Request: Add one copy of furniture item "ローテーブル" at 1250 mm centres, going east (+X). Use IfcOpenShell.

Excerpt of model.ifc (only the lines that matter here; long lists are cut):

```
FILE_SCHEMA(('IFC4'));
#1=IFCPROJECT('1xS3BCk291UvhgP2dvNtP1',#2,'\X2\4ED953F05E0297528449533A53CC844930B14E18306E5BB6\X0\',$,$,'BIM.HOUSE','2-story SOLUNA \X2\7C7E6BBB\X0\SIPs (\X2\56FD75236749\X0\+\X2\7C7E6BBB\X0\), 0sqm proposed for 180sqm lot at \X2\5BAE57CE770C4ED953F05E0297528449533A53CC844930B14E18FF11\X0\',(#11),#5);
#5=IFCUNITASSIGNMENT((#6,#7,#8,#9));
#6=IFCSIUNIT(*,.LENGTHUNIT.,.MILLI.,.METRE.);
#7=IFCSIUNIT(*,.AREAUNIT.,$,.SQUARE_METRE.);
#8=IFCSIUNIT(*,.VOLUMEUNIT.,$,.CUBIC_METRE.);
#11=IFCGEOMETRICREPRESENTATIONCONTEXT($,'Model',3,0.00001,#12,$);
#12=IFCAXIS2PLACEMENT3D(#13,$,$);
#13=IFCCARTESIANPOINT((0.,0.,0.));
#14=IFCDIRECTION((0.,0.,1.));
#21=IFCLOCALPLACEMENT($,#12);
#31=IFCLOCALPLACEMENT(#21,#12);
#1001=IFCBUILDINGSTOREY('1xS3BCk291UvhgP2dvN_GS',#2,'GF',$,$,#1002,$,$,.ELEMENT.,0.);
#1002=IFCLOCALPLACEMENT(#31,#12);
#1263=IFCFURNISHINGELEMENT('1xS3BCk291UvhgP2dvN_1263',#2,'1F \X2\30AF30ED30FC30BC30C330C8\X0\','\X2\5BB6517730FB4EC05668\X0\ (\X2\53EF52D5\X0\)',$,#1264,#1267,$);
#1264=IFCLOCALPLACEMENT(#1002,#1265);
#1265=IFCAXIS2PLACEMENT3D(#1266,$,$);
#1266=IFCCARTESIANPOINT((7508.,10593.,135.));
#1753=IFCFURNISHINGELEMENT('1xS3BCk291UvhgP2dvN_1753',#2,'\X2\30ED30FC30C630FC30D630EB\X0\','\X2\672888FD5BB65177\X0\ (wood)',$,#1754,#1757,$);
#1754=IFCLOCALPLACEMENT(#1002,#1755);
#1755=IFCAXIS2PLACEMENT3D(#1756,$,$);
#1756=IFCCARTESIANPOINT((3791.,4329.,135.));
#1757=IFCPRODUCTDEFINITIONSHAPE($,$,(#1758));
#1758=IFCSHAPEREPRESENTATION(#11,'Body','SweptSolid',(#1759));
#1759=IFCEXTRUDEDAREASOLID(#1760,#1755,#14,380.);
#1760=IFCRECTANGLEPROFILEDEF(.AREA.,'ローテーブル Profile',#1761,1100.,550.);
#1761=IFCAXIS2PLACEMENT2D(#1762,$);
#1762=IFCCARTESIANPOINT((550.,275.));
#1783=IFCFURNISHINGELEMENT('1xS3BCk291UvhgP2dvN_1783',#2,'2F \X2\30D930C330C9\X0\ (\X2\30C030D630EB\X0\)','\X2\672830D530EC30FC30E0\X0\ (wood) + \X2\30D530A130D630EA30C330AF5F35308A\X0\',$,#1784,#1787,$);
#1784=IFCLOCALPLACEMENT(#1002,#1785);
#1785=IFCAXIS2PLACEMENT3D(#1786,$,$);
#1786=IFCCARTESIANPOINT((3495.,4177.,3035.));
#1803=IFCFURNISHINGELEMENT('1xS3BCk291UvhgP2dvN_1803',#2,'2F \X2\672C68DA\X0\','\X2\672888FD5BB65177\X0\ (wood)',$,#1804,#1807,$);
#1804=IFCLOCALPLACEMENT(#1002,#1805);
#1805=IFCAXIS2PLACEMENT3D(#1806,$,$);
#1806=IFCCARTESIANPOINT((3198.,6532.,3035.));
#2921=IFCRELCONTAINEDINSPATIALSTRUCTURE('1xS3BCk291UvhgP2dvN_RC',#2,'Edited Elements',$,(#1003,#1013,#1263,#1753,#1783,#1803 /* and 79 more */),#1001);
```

```python
import numpy as np
import ifcopenshell
import ifcopenshell.api.geometry
import ifcopenshell.api.root
import ifcopenshell.util.element
import ifcopenshell.util.placement

model = ifcopenshell.open("model.ifc")


def reuse_history(source, copy):
    """copy_class also copies each property set's owner history, people and application; keep the originals."""
    for rel in copy.IsDefinedBy:
        if rel.is_a("IfcRelDefinesByProperties") and (history := rel.RelatingPropertyDefinition.OwnerHistory):
            rel.RelatingPropertyDefinition.OwnerHistory = source.OwnerHistory
            ifcopenshell.util.element.remove_deep2(model, history)


source = model.by_guid("1xS3BCk291UvhgP2dvN_1753")
base = ifcopenshell.util.placement.get_local_placement(source.ObjectPlacement)
step = np.array([1.0, 0.0, 0.0]) * 1250.0

for i in range(1, 2):
    copy = ifcopenshell.api.root.copy_class(model, product=source)
    copy.Representation = ifcopenshell.util.element.copy_deep(
        model, source.Representation, exclude=["IfcGeometricRepresentationContext", "IfcRepresentationMap"]
    )
    reuse_history(source, copy)
    matrix = base.copy()
    matrix[:3, 3] += i * step
    print("added at", matrix[:3, 3].round(3) + 0.0)
    ifcopenshell.api.geometry.edit_object_placement(model, product=copy, matrix=matrix, is_si=False)

model.write("model_updated.ifc")
```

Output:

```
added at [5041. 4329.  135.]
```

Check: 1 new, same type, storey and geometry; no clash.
